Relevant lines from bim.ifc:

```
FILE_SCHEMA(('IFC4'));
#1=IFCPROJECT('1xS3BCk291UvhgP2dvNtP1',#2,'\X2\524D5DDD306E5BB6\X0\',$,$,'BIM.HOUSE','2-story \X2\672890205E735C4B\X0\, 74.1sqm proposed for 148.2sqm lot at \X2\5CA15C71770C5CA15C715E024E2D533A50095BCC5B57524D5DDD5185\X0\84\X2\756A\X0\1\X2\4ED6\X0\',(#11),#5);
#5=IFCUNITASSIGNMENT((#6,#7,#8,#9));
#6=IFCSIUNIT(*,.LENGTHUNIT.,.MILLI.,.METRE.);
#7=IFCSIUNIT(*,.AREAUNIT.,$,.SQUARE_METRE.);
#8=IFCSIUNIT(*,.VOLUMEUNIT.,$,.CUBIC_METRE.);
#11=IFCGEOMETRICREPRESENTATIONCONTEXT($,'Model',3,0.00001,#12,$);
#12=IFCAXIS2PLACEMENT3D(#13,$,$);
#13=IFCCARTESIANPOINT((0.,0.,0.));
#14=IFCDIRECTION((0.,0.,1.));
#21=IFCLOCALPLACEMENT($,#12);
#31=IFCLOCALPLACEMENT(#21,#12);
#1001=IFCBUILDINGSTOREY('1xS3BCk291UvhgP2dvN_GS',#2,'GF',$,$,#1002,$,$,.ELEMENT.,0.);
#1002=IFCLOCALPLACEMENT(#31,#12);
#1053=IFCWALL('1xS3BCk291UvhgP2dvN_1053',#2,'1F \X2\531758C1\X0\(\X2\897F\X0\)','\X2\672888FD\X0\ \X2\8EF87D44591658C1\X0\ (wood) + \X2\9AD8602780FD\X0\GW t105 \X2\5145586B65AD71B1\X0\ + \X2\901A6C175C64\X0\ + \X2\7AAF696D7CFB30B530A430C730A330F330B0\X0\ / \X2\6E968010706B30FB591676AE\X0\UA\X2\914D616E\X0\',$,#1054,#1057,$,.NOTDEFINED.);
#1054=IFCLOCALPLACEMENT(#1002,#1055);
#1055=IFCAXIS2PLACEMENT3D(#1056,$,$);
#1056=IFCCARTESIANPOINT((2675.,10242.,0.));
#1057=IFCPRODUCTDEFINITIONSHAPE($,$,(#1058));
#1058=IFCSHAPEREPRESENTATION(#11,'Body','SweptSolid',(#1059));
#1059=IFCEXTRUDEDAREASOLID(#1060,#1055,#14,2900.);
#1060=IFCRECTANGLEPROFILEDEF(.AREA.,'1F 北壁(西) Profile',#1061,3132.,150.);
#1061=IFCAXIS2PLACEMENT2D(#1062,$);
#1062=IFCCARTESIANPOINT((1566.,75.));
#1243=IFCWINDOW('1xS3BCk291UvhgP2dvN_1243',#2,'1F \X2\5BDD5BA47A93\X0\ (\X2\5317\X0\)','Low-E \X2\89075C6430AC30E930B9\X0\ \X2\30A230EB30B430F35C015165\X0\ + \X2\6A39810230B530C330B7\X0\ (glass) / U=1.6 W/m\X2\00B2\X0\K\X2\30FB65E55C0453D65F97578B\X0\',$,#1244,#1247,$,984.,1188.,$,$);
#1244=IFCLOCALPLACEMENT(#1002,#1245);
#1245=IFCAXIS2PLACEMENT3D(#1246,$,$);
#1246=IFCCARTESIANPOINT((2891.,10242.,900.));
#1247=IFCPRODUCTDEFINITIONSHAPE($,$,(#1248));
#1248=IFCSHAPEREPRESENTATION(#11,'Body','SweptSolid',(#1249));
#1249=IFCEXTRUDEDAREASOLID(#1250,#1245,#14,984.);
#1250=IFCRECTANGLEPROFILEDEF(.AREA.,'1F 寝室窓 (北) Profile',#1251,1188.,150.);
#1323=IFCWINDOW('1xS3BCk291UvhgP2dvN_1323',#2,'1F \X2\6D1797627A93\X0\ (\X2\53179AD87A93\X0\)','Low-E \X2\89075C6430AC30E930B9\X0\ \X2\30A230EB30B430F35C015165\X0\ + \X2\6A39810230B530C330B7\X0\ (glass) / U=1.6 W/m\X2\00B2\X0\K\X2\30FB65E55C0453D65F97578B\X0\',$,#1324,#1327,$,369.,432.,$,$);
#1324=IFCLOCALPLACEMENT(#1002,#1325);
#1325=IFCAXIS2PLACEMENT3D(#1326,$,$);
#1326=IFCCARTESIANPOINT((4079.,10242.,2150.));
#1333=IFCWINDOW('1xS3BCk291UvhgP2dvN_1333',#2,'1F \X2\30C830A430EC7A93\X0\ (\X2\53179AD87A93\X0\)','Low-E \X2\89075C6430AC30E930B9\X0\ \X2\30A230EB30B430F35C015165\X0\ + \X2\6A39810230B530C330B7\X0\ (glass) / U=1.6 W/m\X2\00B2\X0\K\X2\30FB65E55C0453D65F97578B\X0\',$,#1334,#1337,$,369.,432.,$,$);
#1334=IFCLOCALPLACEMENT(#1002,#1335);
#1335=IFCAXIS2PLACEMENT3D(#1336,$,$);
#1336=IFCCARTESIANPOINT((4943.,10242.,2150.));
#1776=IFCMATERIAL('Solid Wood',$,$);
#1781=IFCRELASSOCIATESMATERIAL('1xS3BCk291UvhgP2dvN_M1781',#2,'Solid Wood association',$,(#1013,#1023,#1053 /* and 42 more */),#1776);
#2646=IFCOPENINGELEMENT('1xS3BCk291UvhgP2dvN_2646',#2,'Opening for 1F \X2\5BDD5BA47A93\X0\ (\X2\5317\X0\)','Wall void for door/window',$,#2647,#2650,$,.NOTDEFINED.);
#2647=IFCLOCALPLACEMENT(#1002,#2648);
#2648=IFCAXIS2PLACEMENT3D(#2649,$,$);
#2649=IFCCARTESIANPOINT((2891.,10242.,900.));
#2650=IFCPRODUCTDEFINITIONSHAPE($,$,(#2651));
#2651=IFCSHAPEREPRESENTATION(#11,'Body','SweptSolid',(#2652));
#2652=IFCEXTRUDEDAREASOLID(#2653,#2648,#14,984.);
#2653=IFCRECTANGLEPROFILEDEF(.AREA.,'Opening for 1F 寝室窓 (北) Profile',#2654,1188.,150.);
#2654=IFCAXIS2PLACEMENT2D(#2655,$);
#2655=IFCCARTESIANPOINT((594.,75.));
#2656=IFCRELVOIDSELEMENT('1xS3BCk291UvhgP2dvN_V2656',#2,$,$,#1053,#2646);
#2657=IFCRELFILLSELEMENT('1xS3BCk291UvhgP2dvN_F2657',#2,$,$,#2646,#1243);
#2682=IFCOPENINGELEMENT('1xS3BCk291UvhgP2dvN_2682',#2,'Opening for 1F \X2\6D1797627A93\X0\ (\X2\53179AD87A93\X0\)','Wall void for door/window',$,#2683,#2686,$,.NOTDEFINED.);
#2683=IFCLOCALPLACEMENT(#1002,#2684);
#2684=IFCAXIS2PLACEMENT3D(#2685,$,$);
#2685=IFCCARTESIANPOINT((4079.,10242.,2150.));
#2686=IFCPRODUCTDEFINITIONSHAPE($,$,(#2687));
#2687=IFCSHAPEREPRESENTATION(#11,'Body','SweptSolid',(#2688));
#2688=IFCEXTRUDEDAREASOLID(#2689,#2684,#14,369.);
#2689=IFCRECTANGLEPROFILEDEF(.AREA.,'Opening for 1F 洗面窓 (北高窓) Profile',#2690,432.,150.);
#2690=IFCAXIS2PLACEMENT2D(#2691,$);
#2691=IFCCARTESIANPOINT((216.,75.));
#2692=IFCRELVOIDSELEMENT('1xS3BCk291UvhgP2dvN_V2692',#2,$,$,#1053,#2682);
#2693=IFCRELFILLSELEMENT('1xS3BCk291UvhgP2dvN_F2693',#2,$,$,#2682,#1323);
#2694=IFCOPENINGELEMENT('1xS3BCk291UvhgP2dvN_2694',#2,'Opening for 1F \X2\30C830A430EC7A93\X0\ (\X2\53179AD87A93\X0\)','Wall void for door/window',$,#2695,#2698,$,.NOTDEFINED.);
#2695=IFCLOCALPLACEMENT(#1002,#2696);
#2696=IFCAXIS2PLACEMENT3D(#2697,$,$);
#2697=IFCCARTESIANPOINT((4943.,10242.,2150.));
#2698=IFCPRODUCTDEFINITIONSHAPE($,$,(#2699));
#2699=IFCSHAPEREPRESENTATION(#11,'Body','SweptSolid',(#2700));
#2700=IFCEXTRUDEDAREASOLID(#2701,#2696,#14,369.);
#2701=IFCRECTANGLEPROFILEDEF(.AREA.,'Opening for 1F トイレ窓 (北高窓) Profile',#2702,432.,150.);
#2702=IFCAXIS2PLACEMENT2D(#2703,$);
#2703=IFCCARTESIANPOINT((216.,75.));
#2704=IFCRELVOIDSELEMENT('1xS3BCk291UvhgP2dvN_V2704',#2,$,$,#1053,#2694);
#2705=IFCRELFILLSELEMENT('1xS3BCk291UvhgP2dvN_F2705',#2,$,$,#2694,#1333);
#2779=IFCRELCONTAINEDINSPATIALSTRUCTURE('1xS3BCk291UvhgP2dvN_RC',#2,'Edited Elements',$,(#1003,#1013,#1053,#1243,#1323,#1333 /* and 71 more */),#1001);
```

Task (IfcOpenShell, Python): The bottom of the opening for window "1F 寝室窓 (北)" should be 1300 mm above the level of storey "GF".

```python
import numpy as np
import ifcopenshell
import ifcopenshell.api.geometry
import ifcopenshell.geom
import ifcopenshell.util.element
import ifcopenshell.util.placement
import ifcopenshell.util.shape
import ifcopenshell.util.unit

model = ifcopenshell.open("bim.ifc")
unit_scale = ifcopenshell.util.unit.calculate_unit_scale(model)

window = model.by_guid("1xS3BCk291UvhgP2dvN_1243")
opening = window.FillsVoids[0].RelatingOpeningElement
storey = ifcopenshell.util.element.get_container(window, ifc_class="IfcBuildingStorey")
level = ifcopenshell.util.placement.get_local_placement(storey.ObjectPlacement)[2, 3]

# The opening's origin need not be at the sill, so measure its lowest point.
shape = ifcopenshell.geom.create_shape(ifcopenshell.geom.settings(), opening)
bottom = ifcopenshell.util.shape.get_shape_bottom_elevation(shape, shape.geometry) / unit_scale
dz = level + 1.3 / unit_scale - bottom

shift = np.array([0.0, 0.0, dz])
# The window is not placed relative to its opening, so move both.
for product in (opening, window):
    matrix = ifcopenshell.util.placement.get_local_placement(product.ObjectPlacement)
    matrix[:3, 3] += shift
    ifcopenshell.api.geometry.edit_object_placement(model, product=product, matrix=matrix, is_si=False)

print(f"moved by {dz * unit_scale:+.3f} m")

model.write("bim_v2.ifc")
```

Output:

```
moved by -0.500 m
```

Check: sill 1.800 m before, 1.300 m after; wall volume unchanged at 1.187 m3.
